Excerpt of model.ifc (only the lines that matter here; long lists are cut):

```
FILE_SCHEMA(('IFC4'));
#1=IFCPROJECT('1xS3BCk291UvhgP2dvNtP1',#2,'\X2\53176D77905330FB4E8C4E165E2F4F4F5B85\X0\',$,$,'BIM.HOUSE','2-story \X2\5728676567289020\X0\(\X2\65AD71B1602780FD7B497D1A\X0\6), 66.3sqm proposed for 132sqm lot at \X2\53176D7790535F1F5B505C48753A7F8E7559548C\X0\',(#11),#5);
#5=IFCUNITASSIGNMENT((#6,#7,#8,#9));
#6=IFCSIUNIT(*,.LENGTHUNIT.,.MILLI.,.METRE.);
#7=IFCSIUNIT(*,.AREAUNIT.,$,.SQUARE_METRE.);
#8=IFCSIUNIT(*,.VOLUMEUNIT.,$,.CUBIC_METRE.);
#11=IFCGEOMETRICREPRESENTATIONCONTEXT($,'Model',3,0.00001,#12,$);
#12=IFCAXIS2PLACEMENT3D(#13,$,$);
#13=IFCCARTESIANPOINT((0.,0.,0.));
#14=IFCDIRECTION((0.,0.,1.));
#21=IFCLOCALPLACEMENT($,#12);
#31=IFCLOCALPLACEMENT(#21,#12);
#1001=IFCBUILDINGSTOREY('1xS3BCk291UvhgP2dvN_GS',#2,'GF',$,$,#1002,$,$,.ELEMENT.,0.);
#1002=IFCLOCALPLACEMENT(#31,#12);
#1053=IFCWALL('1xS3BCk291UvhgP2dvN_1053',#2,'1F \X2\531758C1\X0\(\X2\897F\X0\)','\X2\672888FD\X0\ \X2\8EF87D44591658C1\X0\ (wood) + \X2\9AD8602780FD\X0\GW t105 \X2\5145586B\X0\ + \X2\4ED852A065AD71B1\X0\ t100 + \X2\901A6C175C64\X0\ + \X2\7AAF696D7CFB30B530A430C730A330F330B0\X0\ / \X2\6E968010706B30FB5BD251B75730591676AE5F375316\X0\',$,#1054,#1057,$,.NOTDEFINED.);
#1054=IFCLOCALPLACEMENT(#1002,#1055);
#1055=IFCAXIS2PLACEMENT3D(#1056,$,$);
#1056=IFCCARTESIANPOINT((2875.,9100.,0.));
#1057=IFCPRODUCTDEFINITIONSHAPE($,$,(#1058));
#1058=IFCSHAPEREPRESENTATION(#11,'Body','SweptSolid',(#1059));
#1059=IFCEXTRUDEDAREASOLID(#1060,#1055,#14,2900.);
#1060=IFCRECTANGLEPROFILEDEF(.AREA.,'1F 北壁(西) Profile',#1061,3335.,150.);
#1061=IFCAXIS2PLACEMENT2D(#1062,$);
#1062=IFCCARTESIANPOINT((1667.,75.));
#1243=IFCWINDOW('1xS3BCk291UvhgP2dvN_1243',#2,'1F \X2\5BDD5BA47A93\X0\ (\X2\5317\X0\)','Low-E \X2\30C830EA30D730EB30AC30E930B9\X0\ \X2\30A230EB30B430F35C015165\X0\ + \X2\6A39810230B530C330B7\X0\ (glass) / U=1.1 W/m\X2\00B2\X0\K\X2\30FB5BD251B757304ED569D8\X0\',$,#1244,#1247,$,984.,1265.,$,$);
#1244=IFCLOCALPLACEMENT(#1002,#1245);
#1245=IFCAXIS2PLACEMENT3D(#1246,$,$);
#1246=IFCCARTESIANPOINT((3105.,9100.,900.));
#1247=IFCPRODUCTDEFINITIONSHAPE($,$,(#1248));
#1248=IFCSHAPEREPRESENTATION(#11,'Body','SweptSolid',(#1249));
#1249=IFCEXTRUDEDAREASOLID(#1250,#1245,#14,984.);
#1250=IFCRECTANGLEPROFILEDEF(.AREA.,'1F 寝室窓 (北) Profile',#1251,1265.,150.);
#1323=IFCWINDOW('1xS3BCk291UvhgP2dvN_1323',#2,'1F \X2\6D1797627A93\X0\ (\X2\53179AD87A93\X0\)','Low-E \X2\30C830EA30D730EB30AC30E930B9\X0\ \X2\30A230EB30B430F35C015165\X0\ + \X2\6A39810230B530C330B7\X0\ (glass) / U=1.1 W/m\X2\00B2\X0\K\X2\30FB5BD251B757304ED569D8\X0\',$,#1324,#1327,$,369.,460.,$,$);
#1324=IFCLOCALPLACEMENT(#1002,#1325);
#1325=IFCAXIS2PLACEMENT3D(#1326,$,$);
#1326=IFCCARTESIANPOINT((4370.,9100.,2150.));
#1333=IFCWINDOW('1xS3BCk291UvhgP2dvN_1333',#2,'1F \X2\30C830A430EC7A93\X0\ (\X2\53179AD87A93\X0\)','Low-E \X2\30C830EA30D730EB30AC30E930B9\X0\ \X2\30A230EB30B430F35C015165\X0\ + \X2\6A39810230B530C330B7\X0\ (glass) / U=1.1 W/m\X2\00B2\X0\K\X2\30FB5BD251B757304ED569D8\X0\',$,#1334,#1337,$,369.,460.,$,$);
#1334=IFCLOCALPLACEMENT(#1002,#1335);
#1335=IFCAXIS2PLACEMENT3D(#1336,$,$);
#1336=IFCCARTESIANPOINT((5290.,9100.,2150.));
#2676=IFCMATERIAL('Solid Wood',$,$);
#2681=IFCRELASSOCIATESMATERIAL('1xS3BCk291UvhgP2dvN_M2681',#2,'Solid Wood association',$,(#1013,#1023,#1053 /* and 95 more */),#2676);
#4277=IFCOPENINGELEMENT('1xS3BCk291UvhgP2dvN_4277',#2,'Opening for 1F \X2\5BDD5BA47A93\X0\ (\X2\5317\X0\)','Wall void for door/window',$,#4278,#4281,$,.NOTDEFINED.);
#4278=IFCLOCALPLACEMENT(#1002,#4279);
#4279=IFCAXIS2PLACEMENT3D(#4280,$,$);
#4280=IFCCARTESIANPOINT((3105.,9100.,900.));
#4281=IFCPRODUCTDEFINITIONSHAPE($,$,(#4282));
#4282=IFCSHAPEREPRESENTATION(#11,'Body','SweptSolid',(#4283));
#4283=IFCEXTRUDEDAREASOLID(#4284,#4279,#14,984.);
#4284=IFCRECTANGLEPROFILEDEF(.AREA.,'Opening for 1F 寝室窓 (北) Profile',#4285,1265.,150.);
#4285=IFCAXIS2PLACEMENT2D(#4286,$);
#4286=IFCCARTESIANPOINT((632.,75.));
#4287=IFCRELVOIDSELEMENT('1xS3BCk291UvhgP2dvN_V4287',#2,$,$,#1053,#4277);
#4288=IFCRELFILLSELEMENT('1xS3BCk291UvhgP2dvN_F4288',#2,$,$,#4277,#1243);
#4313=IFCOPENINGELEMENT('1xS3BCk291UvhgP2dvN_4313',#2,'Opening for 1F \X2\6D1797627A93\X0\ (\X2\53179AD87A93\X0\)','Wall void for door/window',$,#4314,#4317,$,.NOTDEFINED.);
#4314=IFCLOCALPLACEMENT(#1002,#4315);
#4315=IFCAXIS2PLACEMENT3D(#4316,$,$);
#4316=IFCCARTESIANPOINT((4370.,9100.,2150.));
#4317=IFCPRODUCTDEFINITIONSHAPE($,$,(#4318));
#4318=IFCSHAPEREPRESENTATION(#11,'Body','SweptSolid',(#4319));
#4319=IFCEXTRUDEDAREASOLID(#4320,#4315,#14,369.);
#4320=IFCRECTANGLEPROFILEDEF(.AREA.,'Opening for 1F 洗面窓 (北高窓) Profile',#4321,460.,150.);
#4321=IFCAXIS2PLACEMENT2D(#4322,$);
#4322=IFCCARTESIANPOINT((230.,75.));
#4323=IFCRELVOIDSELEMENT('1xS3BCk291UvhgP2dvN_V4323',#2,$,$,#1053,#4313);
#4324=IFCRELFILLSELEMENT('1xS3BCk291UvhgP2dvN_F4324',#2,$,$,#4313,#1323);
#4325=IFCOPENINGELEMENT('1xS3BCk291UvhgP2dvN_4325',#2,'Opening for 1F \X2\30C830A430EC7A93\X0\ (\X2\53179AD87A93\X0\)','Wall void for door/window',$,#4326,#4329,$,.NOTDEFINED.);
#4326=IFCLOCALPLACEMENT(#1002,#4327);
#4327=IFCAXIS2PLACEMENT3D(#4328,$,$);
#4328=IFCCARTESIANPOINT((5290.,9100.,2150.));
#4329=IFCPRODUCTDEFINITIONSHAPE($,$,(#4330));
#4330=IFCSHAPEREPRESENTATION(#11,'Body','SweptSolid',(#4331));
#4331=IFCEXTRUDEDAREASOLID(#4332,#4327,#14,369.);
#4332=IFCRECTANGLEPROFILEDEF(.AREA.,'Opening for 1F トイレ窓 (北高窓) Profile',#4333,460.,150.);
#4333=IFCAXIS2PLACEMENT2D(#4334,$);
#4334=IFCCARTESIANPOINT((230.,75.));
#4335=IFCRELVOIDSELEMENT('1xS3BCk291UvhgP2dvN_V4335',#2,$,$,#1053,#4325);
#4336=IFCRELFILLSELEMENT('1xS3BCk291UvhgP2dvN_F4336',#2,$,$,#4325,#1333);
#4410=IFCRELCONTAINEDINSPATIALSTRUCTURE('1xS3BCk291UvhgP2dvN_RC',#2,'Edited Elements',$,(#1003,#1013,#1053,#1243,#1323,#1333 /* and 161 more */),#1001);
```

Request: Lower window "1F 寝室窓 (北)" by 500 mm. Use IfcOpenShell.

```python
import numpy as np
import ifcopenshell
import ifcopenshell.api.geometry
import ifcopenshell.util.placement
import ifcopenshell.util.unit

model = ifcopenshell.open("model.ifc")
unit_scale = ifcopenshell.util.unit.calculate_unit_scale(model)

window = model.by_guid("1xS3BCk291UvhgP2dvN_1243")
opening = window.FillsVoids[0].RelatingOpeningElement
dz = -0.5 / unit_scale

shift = np.array([0.0, 0.0, dz])
# The window is not placed relative to its opening, so move both.
for product in (opening, window):
    matrix = ifcopenshell.util.placement.get_local_placement(product.ObjectPlacement)
    matrix[:3, 3] += shift
    ifcopenshell.api.geometry.edit_object_placement(model, product=product, matrix=matrix, is_si=False)

print(f"moved by {dz * unit_scale:+.3f} m")

model.write("model-out.ifc")
```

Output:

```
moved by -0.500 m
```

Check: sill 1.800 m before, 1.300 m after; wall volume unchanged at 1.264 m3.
